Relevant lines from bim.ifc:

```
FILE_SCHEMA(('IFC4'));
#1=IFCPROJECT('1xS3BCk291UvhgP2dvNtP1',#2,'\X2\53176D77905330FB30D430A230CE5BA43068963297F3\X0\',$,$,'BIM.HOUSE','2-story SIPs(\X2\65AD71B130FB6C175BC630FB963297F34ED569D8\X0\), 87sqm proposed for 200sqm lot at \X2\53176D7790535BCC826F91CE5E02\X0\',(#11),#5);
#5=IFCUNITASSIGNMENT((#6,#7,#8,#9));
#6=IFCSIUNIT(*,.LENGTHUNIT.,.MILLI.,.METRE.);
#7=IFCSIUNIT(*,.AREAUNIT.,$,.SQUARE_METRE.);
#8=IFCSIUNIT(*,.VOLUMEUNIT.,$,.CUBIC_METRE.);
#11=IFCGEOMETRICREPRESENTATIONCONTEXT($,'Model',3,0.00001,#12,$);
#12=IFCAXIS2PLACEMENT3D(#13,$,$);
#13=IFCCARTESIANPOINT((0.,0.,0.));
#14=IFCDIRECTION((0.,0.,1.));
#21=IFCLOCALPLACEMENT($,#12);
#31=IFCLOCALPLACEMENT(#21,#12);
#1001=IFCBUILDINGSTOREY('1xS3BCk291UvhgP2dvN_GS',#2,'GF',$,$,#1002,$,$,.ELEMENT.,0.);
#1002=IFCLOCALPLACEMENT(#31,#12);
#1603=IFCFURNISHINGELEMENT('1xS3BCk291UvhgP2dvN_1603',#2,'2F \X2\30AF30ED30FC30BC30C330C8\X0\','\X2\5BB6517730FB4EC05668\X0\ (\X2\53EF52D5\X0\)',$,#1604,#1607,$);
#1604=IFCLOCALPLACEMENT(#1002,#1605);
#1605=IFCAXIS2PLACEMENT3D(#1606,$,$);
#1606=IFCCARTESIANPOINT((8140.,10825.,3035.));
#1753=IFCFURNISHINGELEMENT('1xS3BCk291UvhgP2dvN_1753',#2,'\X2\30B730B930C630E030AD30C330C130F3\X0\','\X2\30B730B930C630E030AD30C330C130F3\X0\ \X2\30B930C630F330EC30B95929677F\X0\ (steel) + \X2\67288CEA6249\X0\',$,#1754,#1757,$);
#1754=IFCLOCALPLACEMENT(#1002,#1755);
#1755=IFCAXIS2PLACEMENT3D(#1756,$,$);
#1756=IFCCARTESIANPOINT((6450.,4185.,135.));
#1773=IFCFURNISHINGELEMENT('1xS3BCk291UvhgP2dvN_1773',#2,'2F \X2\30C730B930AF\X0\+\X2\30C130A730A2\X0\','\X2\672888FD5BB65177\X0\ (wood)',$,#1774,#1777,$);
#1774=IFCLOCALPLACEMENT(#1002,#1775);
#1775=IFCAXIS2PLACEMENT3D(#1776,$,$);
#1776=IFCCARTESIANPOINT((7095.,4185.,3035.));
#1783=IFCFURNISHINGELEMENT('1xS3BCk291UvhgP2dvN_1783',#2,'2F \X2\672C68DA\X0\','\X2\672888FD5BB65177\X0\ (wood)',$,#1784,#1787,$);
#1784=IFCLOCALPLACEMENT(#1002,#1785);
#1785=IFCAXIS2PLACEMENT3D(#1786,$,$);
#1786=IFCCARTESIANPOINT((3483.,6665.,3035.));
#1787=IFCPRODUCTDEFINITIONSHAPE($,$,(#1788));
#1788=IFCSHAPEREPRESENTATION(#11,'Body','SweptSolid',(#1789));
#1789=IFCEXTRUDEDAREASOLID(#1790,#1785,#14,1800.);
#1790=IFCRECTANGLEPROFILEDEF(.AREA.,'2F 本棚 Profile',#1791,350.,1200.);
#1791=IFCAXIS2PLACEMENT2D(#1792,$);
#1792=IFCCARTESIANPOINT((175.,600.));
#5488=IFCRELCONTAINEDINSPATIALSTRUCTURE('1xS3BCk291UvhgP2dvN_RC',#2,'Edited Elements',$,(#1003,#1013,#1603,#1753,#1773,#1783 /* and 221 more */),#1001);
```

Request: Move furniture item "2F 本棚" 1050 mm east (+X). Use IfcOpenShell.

```python
import ifcopenshell
import ifcopenshell.api.geometry
import ifcopenshell.util.placement
import ifcopenshell.util.unit

model = ifcopenshell.open("bim.ifc")
unit_scale = ifcopenshell.util.unit.calculate_unit_scale(model)

item = model.by_guid("1xS3BCk291UvhgP2dvN_1783")
matrix = ifcopenshell.util.placement.get_local_placement(item.ObjectPlacement)
matrix[0, 3] += 1.05 / unit_scale
ifcopenshell.api.geometry.edit_object_placement(model, product=item, matrix=matrix, is_si=False)

print(ifcopenshell.util.placement.get_local_placement(item.ObjectPlacement).round(3) + 0.0)

model.write("bim_rev.ifc")
```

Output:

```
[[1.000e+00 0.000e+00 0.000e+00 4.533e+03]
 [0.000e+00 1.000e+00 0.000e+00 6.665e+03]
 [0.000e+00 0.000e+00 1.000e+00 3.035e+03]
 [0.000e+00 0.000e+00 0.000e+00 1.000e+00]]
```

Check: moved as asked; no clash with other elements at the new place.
